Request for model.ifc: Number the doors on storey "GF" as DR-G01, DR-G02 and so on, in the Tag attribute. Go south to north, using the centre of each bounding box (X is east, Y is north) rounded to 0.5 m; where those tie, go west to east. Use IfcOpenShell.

First a look at what the model holds.

```python
import ifcopenshell
import ifcopenshell.util.element
import ifcopenshell.util.placement

model = ifcopenshell.open("model.ifc")
print(model.schema)
storey = next(s for s in model.by_type("IfcBuildingStorey") if s.Name == "GF")
doors = [e for e in ifcopenshell.util.element.get_decomposition(storey) if e.is_a("IfcDoor")]
for e in sorted(doors, key=lambda e: e.id()):
    origin = ifcopenshell.util.placement.get_local_placement(e.ObjectPlacement)[:3, 3]
    print(e.id(), e.Tag, e.Name, origin.round(2) + 0.0, sep=" | ")
```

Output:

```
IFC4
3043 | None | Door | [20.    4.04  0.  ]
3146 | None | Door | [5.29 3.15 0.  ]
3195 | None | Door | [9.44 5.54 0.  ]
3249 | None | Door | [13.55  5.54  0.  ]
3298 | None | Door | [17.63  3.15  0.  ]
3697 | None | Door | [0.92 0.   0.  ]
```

```python
import ifcopenshell
import ifcopenshell.geom
import ifcopenshell.util.element
import ifcopenshell.util.shape

model = ifcopenshell.open("model.ifc")
settings = ifcopenshell.geom.settings()
settings.set("use-world-coords", True)


def centre(element):
    shape = ifcopenshell.geom.create_shape(settings, element)
    return ifcopenshell.util.shape.get_bbox_centroid(shape.geometry)


storey = next(s for s in model.by_type("IfcBuildingStorey") if s.Name == "GF")
doors = [e for e in ifcopenshell.util.element.get_decomposition(storey) if e.is_a("IfcDoor")]

# Insertion points can sit at a corner or the storey origin, so sort by the geometry (in metres).
centres = {e: centre(e) for e in doors}
doors.sort(key=lambda e: (round(centres[e][1] / 0.5), centres[e][0]))

for i, e in enumerate(doors, start=1):
    number = f"DR-G{i:02d}"
    e.Tag = number
    print(e.id(), number)

model.write("model_rev.ifc")
```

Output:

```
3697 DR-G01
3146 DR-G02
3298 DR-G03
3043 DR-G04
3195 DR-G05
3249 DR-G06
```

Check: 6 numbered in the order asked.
